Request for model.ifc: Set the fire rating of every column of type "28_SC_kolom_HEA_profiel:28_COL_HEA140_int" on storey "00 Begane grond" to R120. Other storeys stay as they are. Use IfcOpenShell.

First a look at what the model holds.

```python
import ifcopenshell
import ifcopenshell.util.element

model = ifcopenshell.open("model.ifc")
print(model.schema)
storey = next(s for s in model.by_type("IfcBuildingStorey") if s.Name == "00 Begane grond")
columns = [e for e in ifcopenshell.util.element.get_decomposition(storey) if e.is_a("IfcColumn")]
seen = {}
for e in columns:
    element_type = ifcopenshell.util.element.get_type(e)
    key = (element_type.Name if element_type != e and element_type else None, ifcopenshell.util.element.get_pset(e, "Pset_ColumnCommon", "FireRating"))
    seen[key] = seen.get(key, 0) + 1
for (name, value), count in sorted(seen.items(), key=str):
    print(count, "x", name, "|", value)
```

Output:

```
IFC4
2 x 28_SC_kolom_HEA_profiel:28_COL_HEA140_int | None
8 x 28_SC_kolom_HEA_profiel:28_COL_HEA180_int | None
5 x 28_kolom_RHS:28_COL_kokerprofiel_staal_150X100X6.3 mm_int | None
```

```python
import ifcopenshell
import ifcopenshell.api.pset
import ifcopenshell.util.element

model = ifcopenshell.open("model.ifc")

storey = next(s for s in model.by_type("IfcBuildingStorey") if s.Name == "00 Begane grond")
columns = [e for e in ifcopenshell.util.element.get_decomposition(storey) if e.is_a("IfcColumn")]

count = 0
for e in columns:
    element_type = ifcopenshell.util.element.get_type(e)
    if element_type in (None, e) or element_type.Name != "28_SC_kolom_HEA_profiel:28_COL_HEA140_int":
        continue
    # add_pset returns the element's existing set when there is one.
    pset = ifcopenshell.api.pset.add_pset(model, product=e, name="Pset_ColumnCommon")
    ifcopenshell.api.pset.edit_pset(model, pset=pset, properties={"FireRating": "R120"})
    count += 1

print(count, "columns updated")

model.write("model-out.ifc")
```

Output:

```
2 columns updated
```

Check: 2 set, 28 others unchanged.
